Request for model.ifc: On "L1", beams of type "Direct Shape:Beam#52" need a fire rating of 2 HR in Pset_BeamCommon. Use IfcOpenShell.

First a look at what the model holds.

```python
import ifcopenshell
import ifcopenshell.util.element

model = ifcopenshell.open("model.ifc")
print(model.schema)
storey = next(s for s in model.by_type("IfcBuildingStorey") if s.Name == "L1")
beams = [e for e in ifcopenshell.util.element.get_decomposition(storey) if e.is_a("IfcBeam")]
seen = {}
for e in beams:
    element_type = ifcopenshell.util.element.get_type(e)
    key = (element_type.Name if element_type != e and element_type else None, ifcopenshell.util.element.get_pset(e, "Pset_BeamCommon", "FireRating"))
    seen[key] = seen.get(key, 0) + 1
for (name, value), count in sorted(seen.items(), key=str):
    print(count, "x", name, "|", value)
```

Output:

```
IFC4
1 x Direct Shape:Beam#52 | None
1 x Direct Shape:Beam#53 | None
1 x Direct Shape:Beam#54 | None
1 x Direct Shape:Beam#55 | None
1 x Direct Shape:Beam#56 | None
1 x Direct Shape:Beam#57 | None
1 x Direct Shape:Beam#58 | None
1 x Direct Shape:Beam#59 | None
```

```python
import ifcopenshell
import ifcopenshell.api.pset
import ifcopenshell.util.element

model = ifcopenshell.open("model.ifc")

storey = next(s for s in model.by_type("IfcBuildingStorey") if s.Name == "L1")
beams = [e for e in ifcopenshell.util.element.get_decomposition(storey) if e.is_a("IfcBeam")]

count = 0
for e in beams:
    element_type = ifcopenshell.util.element.get_type(e)
    if element_type in (None, e) or element_type.Name != "Direct Shape:Beam#52":
        continue
    # add_pset returns the element's existing set when there is one.
    pset = ifcopenshell.api.pset.add_pset(model, product=e, name="Pset_BeamCommon")
    ifcopenshell.api.pset.edit_pset(model, pset=pset, properties={"FireRating": "2 HR"})
    count += 1

print(count, "beams updated")

model.write("model_rev.ifc")
```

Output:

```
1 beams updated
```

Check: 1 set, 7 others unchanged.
